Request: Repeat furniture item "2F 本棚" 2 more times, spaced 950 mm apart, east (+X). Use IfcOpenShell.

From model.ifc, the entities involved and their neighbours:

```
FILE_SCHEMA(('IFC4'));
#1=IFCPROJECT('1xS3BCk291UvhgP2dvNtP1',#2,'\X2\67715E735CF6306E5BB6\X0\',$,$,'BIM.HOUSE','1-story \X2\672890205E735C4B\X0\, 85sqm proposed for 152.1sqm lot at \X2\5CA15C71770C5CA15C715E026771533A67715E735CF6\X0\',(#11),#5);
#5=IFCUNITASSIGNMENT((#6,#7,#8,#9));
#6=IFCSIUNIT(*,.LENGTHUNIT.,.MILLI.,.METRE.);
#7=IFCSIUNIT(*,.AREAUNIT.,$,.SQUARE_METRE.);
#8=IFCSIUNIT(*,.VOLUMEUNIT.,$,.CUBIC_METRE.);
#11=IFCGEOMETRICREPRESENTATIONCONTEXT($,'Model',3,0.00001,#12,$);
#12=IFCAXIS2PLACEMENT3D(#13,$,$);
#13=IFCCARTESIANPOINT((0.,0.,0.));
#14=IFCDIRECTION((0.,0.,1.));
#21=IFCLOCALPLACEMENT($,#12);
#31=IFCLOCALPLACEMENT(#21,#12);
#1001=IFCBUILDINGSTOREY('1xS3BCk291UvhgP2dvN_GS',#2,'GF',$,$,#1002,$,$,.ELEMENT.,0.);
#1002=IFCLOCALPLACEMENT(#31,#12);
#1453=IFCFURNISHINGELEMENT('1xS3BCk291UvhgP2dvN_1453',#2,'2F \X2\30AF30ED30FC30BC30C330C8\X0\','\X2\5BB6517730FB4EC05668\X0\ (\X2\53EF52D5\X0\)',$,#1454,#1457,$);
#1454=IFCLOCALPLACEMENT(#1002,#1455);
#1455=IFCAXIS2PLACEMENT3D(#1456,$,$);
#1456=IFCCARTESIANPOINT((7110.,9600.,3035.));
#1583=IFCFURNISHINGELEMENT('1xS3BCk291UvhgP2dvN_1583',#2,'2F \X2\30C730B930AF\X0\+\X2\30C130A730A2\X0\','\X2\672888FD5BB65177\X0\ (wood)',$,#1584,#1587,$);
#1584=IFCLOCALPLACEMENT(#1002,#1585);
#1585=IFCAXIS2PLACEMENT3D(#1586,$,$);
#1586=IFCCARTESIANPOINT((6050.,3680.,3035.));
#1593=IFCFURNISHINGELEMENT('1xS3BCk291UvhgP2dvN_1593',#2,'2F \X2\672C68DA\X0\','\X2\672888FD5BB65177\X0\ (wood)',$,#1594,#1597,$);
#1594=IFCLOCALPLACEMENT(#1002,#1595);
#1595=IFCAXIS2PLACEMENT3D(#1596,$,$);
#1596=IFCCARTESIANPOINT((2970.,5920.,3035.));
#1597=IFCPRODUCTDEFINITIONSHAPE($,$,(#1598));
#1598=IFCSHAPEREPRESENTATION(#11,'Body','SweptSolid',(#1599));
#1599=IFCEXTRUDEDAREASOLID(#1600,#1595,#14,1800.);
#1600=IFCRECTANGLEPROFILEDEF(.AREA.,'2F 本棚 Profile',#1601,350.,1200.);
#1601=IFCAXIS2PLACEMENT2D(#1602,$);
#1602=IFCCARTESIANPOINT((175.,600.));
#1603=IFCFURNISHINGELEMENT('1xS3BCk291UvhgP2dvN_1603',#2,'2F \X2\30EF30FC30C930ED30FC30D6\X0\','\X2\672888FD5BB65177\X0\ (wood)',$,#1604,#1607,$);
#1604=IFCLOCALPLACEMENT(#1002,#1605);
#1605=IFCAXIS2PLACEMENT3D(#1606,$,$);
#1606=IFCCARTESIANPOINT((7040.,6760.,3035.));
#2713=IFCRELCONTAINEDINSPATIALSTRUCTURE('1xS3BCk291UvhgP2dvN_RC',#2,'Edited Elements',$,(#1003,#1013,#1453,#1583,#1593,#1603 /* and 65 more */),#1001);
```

```python
import numpy as np
import ifcopenshell
import ifcopenshell.api.geometry
import ifcopenshell.api.root
import ifcopenshell.util.element
import ifcopenshell.util.placement
import ifcopenshell.util.unit

model = ifcopenshell.open("model.ifc")
unit_scale = ifcopenshell.util.unit.calculate_unit_scale(model)


def reuse_history(source, copy):
    """copy_class also copies each property set's owner history, people and application; keep the originals."""
    for rel in copy.IsDefinedBy:
        if rel.is_a("IfcRelDefinesByProperties") and (history := rel.RelatingPropertyDefinition.OwnerHistory):
            rel.RelatingPropertyDefinition.OwnerHistory = source.OwnerHistory
            ifcopenshell.util.element.remove_deep2(model, history)


source = model.by_id(1593)
base = ifcopenshell.util.placement.get_local_placement(source.ObjectPlacement)
step = np.array([1.0, 0.0, 0.0]) * 0.95 / unit_scale

for i in range(1, 3):
    copy = ifcopenshell.api.root.copy_class(model, product=source)
    copy.Representation = ifcopenshell.util.element.copy_deep(
        model, source.Representation, exclude=["IfcGeometricRepresentationContext", "IfcRepresentationMap"]
    )
    reuse_history(source, copy)
    matrix = base.copy()
    matrix[:3, 3] += i * step
    print("added at", matrix[:3, 3].round(3) + 0.0)
    ifcopenshell.api.geometry.edit_object_placement(model, product=copy, matrix=matrix, is_si=False)

model.write("model_updated.ifc")
```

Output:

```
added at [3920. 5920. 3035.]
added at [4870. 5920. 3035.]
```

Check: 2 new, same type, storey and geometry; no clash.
